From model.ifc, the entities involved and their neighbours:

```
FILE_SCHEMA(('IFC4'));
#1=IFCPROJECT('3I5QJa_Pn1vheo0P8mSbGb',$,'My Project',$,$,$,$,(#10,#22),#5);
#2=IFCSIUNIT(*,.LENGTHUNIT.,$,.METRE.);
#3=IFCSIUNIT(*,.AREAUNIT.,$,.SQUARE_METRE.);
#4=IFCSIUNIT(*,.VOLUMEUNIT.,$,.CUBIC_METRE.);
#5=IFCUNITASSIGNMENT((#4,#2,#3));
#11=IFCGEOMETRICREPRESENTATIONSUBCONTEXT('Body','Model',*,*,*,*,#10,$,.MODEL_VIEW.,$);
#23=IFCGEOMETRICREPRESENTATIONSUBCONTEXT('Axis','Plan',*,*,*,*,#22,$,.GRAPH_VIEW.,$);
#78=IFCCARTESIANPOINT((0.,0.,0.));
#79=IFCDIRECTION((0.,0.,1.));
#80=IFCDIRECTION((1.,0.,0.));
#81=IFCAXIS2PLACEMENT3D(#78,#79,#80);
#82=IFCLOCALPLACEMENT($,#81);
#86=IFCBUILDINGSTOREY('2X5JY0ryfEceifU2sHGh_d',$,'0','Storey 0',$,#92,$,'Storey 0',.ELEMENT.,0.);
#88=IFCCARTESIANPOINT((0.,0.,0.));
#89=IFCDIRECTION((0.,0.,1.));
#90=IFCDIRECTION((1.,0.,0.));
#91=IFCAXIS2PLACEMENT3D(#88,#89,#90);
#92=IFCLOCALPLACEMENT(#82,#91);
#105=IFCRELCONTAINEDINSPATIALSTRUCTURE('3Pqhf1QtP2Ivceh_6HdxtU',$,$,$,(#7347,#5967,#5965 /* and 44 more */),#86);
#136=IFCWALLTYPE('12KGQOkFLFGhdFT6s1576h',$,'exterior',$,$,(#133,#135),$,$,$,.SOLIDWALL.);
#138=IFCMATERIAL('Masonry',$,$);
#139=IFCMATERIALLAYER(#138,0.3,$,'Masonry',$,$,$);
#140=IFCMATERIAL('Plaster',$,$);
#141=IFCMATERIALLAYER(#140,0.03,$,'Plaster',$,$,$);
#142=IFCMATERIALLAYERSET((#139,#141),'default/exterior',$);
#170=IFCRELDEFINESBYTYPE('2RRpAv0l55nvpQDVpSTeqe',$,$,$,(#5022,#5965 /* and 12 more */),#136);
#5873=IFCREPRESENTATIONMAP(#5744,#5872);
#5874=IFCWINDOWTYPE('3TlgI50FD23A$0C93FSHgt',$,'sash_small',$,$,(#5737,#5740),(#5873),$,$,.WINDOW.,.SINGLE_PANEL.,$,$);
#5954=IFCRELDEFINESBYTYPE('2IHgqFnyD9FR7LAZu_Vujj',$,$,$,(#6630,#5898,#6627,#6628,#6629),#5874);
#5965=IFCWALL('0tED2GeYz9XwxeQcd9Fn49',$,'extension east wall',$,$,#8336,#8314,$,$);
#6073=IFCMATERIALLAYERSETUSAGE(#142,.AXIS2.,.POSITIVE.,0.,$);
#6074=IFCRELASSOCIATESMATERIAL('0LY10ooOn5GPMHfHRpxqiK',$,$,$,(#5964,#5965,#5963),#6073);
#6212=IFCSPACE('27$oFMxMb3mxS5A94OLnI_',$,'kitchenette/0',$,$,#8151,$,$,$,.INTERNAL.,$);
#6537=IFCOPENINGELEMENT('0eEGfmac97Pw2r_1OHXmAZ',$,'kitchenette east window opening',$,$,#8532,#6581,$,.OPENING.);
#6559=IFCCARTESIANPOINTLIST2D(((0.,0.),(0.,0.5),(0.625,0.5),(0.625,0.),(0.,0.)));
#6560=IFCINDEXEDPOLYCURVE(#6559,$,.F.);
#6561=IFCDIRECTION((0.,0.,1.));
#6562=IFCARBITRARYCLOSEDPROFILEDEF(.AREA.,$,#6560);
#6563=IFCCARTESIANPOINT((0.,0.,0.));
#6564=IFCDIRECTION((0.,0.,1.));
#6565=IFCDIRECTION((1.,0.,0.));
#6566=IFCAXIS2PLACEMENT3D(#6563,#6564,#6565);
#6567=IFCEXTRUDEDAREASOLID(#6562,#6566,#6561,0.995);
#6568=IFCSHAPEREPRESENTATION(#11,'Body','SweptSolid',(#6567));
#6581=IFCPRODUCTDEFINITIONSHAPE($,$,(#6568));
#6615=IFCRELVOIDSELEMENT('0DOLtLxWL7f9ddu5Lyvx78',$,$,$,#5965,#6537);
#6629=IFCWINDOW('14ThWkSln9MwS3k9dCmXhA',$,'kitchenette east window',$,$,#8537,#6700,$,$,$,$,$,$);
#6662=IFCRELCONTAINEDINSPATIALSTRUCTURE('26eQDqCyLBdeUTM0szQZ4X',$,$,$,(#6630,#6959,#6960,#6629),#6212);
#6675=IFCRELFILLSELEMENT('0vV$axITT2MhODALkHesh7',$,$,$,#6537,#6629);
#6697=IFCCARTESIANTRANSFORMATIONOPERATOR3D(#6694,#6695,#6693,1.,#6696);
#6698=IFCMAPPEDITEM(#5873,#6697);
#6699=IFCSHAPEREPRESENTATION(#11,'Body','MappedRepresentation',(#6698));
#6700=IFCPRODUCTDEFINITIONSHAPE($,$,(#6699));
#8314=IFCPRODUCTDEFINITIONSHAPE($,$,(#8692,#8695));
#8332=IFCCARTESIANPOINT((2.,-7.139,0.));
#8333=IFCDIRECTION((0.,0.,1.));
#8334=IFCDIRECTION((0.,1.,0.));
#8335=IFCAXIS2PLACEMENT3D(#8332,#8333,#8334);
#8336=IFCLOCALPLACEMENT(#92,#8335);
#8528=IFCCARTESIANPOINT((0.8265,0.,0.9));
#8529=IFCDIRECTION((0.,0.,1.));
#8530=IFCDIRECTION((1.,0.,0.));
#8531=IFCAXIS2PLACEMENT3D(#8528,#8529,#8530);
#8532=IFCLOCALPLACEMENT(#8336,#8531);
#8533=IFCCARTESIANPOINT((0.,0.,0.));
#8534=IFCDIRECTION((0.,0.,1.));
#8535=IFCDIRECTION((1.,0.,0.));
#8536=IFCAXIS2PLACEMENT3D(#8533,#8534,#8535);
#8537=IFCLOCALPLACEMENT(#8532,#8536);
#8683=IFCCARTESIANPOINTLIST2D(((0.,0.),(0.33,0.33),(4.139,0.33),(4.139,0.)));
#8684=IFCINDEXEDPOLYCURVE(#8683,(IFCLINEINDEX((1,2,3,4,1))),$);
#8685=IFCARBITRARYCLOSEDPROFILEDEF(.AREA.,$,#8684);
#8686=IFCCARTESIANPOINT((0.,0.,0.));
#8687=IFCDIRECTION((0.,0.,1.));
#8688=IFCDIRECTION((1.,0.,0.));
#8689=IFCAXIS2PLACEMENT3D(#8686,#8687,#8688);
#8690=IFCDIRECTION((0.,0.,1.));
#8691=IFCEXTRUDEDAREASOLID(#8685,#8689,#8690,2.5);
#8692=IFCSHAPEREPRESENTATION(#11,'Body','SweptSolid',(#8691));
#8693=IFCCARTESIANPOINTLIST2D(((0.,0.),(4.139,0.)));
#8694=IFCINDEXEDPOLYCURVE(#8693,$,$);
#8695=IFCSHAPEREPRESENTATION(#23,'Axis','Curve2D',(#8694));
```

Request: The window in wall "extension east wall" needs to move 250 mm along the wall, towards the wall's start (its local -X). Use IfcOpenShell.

```python
import ifcopenshell
import ifcopenshell.api.geometry
import ifcopenshell.util.placement
import ifcopenshell.util.unit

model = ifcopenshell.open("model.ifc")
unit_scale = ifcopenshell.util.unit.calculate_unit_scale(model)

window = model.by_guid("14ThWkSln9MwS3k9dCmXhA")
opening = window.FillsVoids[0].RelatingOpeningElement
wall = opening.VoidsElements[0].RelatingBuildingElement

wall_matrix = ifcopenshell.util.placement.get_local_placement(wall.ObjectPlacement)
shift = wall_matrix[:3, 0] * -0.25 / unit_scale
before = ifcopenshell.util.placement.get_local_placement(window.ObjectPlacement)[:3, 3].copy()

# The window is placed relative to its opening, so it follows when the opening moves.
matrix = ifcopenshell.util.placement.get_local_placement(opening.ObjectPlacement)
matrix[:3, 3] += shift
ifcopenshell.api.geometry.edit_object_placement(
    model, product=opening, matrix=matrix, is_si=False, should_transform_children=True
)

after = ifcopenshell.util.placement.get_local_placement(window.ObjectPlacement)[:3, 3]
print("window moved by", (after - before).round(3) + 0.0)

model.write("model_rev.ifc")
```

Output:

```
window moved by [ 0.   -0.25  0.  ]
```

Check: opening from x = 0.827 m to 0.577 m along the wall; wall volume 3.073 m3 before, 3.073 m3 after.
